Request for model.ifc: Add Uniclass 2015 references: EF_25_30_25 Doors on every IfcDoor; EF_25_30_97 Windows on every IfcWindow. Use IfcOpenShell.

First a look at what the model holds.

```python
import ifcopenshell

model = ifcopenshell.open("model.ifc")
print(model.schema)
print("classifications:", [c.Name for c in model.by_type("IfcClassification")])
for ifc_class in ("IfcDoor", "IfcRoof", "IfcStair", "IfcWall", "IfcWindow"):
    print(ifc_class, len(model.by_type(ifc_class)))
```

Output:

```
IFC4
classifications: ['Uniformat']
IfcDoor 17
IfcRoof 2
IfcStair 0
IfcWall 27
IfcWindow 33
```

```python
import ifcopenshell
import ifcopenshell.api.classification

model = ifcopenshell.open("model.ifc")

system = ifcopenshell.api.classification.add_classification(model, classification="Uniclass 2015")

codes = {
    "IfcDoor": ("EF_25_30_25", "Doors"),
    "IfcWindow": ("EF_25_30_97", "Windows"),
}
for ifc_class, (code, name) in codes.items():
    products = model.by_type(ifc_class)
    ifcopenshell.api.classification.add_reference(
        model, products=products, classification=system, identification=code, name=name
    )
    print(code, len(products))

model.write("model_updated.ifc")
```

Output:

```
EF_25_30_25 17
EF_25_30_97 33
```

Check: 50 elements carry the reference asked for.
